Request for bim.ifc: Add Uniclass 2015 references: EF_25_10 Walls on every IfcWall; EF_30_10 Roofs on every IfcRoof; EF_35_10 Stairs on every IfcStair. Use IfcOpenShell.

First a look at what the model holds.

```python
import ifcopenshell

model = ifcopenshell.open("bim.ifc")
print(model.schema)
print("classifications:", [c.Name for c in model.by_type("IfcClassification")])
for ifc_class in ("IfcDoor", "IfcRoof", "IfcStair", "IfcWall", "IfcWindow"):
    print(ifc_class, len(model.by_type(ifc_class)))
```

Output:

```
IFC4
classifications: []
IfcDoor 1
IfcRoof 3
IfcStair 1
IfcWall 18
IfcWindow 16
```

```python
import ifcopenshell
import ifcopenshell.api.classification

model = ifcopenshell.open("bim.ifc")

system = ifcopenshell.api.classification.add_classification(model, classification="Uniclass 2015")

codes = {
    "IfcWall": ("EF_25_10", "Walls"),
    "IfcRoof": ("EF_30_10", "Roofs"),
    "IfcStair": ("EF_35_10", "Stairs"),
}
for ifc_class, (code, name) in codes.items():
    products = model.by_type(ifc_class)
    ifcopenshell.api.classification.add_reference(
        model, products=products, classification=system, identification=code, name=name
    )
    print(code, len(products))

model.write("bim-out.ifc")
```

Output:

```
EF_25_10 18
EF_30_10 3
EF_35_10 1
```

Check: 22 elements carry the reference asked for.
